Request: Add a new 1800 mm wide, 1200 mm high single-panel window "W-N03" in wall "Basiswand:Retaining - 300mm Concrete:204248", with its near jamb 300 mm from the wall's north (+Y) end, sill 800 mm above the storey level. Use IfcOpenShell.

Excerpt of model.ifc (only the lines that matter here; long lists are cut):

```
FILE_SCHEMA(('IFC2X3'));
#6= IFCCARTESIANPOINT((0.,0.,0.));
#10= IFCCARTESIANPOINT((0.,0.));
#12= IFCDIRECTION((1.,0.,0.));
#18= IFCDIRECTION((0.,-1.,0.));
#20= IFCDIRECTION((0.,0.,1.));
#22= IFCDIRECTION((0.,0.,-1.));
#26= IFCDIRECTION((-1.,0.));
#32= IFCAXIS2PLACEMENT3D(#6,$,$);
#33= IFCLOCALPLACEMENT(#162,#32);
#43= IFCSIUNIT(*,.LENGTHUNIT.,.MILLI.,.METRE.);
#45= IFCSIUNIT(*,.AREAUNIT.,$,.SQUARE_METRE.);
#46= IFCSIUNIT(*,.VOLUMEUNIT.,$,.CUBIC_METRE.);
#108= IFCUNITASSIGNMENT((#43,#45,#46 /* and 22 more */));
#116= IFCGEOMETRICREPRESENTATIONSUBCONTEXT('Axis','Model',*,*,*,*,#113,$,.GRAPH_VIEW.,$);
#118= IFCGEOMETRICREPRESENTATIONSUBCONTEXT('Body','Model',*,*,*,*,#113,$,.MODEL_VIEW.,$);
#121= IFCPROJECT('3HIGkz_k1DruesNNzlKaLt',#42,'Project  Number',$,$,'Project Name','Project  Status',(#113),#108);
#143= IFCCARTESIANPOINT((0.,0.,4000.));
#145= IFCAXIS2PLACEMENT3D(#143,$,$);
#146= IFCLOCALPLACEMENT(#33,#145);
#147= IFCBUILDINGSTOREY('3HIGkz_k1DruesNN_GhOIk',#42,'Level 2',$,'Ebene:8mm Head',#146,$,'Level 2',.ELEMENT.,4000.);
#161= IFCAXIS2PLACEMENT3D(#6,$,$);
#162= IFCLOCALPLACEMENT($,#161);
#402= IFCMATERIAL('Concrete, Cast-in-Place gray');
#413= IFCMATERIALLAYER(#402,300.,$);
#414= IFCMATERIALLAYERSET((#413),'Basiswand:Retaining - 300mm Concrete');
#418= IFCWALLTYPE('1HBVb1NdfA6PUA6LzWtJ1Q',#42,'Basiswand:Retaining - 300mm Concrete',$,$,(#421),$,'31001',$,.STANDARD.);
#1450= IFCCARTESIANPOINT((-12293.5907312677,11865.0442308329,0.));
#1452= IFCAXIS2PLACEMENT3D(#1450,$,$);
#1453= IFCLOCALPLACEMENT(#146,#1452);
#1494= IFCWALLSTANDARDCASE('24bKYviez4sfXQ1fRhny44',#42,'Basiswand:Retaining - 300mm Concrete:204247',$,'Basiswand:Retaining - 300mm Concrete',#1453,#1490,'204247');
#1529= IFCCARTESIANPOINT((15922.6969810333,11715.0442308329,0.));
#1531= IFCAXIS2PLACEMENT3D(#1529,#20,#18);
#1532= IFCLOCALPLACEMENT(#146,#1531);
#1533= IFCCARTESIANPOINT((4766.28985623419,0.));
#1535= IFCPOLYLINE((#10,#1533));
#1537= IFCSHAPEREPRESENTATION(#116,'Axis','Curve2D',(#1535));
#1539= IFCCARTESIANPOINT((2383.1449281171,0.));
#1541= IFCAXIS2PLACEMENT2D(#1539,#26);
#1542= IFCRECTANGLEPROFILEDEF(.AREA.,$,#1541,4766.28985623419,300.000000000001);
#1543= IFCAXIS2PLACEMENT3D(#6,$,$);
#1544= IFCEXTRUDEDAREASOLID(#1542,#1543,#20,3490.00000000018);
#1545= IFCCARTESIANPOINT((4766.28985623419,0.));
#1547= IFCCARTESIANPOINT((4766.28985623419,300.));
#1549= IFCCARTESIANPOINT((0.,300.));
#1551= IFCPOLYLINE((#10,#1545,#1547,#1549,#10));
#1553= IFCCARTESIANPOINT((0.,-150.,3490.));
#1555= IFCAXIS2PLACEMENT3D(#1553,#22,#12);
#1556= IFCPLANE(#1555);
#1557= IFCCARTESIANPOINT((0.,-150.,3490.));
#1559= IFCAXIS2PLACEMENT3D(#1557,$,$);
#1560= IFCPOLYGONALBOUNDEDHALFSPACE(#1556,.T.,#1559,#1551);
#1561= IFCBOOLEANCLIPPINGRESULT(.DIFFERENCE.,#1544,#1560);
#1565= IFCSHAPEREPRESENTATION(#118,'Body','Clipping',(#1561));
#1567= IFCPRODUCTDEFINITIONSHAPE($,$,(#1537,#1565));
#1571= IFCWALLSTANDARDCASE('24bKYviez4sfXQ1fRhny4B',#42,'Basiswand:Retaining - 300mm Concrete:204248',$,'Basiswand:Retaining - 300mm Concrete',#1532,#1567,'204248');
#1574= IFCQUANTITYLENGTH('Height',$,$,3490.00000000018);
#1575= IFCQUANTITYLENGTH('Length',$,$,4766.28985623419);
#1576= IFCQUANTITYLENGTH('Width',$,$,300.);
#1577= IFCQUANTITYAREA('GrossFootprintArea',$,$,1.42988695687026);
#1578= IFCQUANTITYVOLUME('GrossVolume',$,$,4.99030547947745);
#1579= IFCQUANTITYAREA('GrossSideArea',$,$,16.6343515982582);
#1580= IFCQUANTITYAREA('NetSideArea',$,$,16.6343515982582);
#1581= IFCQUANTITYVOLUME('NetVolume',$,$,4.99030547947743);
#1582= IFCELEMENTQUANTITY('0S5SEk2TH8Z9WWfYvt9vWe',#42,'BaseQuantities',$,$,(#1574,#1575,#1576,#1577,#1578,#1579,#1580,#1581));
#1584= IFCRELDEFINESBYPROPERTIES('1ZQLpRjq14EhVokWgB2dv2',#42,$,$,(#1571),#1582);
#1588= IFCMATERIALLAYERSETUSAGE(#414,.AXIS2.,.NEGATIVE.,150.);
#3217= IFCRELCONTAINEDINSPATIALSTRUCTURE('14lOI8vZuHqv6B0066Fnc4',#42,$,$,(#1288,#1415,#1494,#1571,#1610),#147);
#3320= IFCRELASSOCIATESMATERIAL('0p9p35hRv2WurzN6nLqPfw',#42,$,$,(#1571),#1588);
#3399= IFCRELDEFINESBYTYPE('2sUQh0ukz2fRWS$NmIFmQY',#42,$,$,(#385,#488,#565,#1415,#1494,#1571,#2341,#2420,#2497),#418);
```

```python
import numpy as np
import ifcopenshell
import ifcopenshell.api.feature
import ifcopenshell.api.geometry
import ifcopenshell.api.pset
import ifcopenshell.api.root
import ifcopenshell.api.spatial
import ifcopenshell.api.type
import ifcopenshell.geom
import ifcopenshell.util.element
import ifcopenshell.util.placement
import ifcopenshell.util.representation
import ifcopenshell.util.shape
import ifcopenshell.util.unit

model = ifcopenshell.open("model.ifc")
unit_scale = ifcopenshell.util.unit.calculate_unit_scale(model)
area_scale = ifcopenshell.util.unit.calculate_unit_scale(model, "AREAUNIT")
volume_scale = ifcopenshell.util.unit.calculate_unit_scale(model, "VOLUMEUNIT")
settings = ifcopenshell.geom.settings()


def volume(element):
    """Net volume in cubic metres, openings subtracted."""
    shape = ifcopenshell.geom.create_shape(settings, element)
    return ifcopenshell.util.shape.get_volume(shape.geometry)


wall = model.by_id(1571)
storey = ifcopenshell.util.element.get_container(wall, ifc_class="IfcBuildingStorey")
context = ifcopenshell.util.representation.get_context(model, "Model", "Body", "MODEL_VIEW")
before = volume(wall)

width, height, from_end, sill = 1.8, 1.2, 0.3, 0.8  # metres

# The wall runs along its own X axis, and the end named is its -X end.
wall_shape = ifcopenshell.geom.create_shape(settings, wall)
x, y, z = ifcopenshell.util.shape.get_vertices(wall_shape.geometry).T
start = x.min() + from_end
face, thickness = float(y.min()), float(y.max() - y.min())
wall_matrix = ifcopenshell.util.placement.get_local_placement(wall.ObjectPlacement)
level = ifcopenshell.util.placement.get_local_placement(storey.ObjectPlacement)[2, 3]


def in_wall(x, y):
    """Placement at x, y metres in the wall's axes, at sill height."""
    matrix = wall_matrix.copy()
    matrix[:, 3] = wall_matrix @ np.array([x / unit_scale, y / unit_scale, 0.0, 1.0])
    matrix[2, 3] = level + sill / unit_scale
    return matrix


# Opening: a box that overshoots both wall faces by 50 mm.
opening = ifcopenshell.api.root.create_entity(model, ifc_class="IfcOpeningElement")
box = ifcopenshell.api.geometry.add_wall_representation(
    model, context=context, length=width, height=height, thickness=thickness + 0.1
)
ifcopenshell.api.geometry.assign_representation(model, product=opening, representation=box)
ifcopenshell.api.geometry.edit_object_placement(model, product=opening, matrix=in_wall(start, face - 0.05), is_si=False)
ifcopenshell.api.feature.add_feature(model, feature=opening, element=wall)

window = ifcopenshell.api.root.create_entity(model, ifc_class="IfcWindow", name="W-N03")
window.OverallWidth, window.OverallHeight = width / unit_scale, height / unit_scale
body = ifcopenshell.api.geometry.add_window_representation(
    model,
    context=context,
    overall_width=window.OverallWidth,
    overall_height=window.OverallHeight,
    partition_type="SINGLE_PANEL",
)
ifcopenshell.api.geometry.assign_representation(model, product=window, representation=body)
ifcopenshell.api.spatial.assign_container(model, products=[window], relating_structure=storey)
fills = ifcopenshell.api.feature.add_filling(model, opening=opening, element=window)
fills.OwnerHistory = window.OwnerHistory  # required in IFC2X3

# IFC2X3 keeps the operation on the window style.
style = ifcopenshell.api.root.create_entity(model, ifc_class="IfcWindowStyle", name="W-N03")
style.OperationType, style.ConstructionType = "SINGLE_PANEL", "NOTDEFINED"
style.ParameterTakesPrecedence = style.Sizeable = False
ifcopenshell.api.type.assign_type(model, related_objects=[window], relating_type=style)

# Centre the window in the wall's thickness.
ifcopenshell.api.geometry.edit_object_placement(model, product=window, matrix=in_wall(start, face), is_si=False)
window_shape = ifcopenshell.geom.create_shape(settings, window)
depth = ifcopenshell.util.shape.get_vertices(window_shape.geometry)[:, 1]
offset = face + thickness / 2 - (depth.min() + depth.max()) / 2
ifcopenshell.api.geometry.edit_object_placement(model, product=window, matrix=in_wall(start, offset), is_si=False)

after = volume(wall)

# Update the wall's stored quantities.
qto = model.by_id(ifcopenshell.util.element.get_pset(wall, "BaseQuantities", should_inherit=False)["id"])
ifcopenshell.api.pset.edit_qto(model, qto=qto, properties={
    "NetSideArea": after / thickness / area_scale,
    "NetVolume": after / volume_scale,
})

print(f"wall volume {before:.3f} -> {after:.3f} m3")

model.write("model_rev.ifc")
```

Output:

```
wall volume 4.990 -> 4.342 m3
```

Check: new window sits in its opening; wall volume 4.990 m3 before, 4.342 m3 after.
